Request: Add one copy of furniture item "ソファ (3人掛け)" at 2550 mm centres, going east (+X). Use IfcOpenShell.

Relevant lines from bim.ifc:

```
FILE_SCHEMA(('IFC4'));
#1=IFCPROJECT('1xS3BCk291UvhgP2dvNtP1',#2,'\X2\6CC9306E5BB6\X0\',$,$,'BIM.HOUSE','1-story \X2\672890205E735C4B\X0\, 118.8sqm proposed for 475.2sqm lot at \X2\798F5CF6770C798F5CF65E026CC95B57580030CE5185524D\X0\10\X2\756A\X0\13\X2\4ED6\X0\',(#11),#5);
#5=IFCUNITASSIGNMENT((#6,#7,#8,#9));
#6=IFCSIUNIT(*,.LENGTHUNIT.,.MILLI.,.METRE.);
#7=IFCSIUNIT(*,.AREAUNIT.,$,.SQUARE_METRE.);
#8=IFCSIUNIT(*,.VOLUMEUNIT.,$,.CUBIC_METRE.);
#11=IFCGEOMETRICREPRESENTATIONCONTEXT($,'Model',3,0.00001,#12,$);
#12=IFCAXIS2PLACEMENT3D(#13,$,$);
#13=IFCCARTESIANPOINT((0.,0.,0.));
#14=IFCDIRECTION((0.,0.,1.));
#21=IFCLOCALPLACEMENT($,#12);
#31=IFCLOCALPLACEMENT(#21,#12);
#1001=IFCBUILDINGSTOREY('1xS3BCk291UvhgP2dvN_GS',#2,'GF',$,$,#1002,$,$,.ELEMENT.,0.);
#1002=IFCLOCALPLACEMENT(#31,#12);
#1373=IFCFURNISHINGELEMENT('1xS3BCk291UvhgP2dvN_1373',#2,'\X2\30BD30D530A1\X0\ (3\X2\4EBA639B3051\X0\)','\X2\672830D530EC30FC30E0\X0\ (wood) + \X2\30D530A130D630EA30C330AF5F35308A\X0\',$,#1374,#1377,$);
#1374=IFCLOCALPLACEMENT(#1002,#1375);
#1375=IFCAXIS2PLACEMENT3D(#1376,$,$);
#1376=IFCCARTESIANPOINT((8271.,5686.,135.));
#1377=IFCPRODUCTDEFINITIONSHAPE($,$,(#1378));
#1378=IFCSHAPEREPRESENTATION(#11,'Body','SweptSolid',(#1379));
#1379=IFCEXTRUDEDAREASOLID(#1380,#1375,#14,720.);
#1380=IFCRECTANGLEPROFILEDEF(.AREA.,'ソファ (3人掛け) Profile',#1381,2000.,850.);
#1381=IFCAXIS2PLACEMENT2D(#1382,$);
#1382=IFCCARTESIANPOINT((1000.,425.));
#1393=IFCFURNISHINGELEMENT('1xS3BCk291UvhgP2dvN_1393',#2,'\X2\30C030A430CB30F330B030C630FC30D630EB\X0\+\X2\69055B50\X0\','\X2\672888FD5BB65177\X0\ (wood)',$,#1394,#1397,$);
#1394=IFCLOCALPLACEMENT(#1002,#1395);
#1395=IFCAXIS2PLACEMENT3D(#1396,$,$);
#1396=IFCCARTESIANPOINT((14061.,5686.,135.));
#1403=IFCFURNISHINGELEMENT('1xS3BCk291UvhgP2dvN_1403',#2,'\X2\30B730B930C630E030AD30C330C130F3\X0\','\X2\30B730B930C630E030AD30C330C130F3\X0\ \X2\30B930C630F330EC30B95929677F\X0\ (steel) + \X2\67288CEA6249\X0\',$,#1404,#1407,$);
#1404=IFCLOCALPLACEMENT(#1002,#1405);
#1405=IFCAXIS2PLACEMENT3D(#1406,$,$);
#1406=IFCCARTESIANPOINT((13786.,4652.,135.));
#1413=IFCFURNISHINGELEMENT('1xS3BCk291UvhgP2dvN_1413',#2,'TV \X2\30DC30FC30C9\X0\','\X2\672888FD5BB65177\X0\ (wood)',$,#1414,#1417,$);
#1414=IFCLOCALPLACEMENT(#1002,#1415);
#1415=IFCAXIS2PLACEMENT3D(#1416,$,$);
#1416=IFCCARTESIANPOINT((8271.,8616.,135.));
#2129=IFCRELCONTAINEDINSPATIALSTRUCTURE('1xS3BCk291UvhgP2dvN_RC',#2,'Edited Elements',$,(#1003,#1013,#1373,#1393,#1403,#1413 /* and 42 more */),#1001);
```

```python
import numpy as np
import ifcopenshell
import ifcopenshell.api.geometry
import ifcopenshell.api.root
import ifcopenshell.util.element
import ifcopenshell.util.placement

model = ifcopenshell.open("bim.ifc")


def reuse_history(source, copy):
    """copy_class also copies each property set's owner history, people and application; keep the originals."""
    for rel in copy.IsDefinedBy:
        if rel.is_a("IfcRelDefinesByProperties") and (history := rel.RelatingPropertyDefinition.OwnerHistory):
            rel.RelatingPropertyDefinition.OwnerHistory = source.OwnerHistory
            ifcopenshell.util.element.remove_deep2(model, history)


source = model.by_guid("1xS3BCk291UvhgP2dvN_1373")
base = ifcopenshell.util.placement.get_local_placement(source.ObjectPlacement)
step = np.array([1.0, 0.0, 0.0]) * 2550.0

for i in range(1, 2):
    copy = ifcopenshell.api.root.copy_class(model, product=source)
    copy.Representation = ifcopenshell.util.element.copy_deep(
        model, source.Representation, exclude=["IfcGeometricRepresentationContext", "IfcRepresentationMap"]
    )
    reuse_history(source, copy)
    matrix = base.copy()
    matrix[:3, 3] += i * step
    print("added at", matrix[:3, 3].round(3) + 0.0)
    ifcopenshell.api.geometry.edit_object_placement(model, product=copy, matrix=matrix, is_si=False)

model.write("bim_edited.ifc")
```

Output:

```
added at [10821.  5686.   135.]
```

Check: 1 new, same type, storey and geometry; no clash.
